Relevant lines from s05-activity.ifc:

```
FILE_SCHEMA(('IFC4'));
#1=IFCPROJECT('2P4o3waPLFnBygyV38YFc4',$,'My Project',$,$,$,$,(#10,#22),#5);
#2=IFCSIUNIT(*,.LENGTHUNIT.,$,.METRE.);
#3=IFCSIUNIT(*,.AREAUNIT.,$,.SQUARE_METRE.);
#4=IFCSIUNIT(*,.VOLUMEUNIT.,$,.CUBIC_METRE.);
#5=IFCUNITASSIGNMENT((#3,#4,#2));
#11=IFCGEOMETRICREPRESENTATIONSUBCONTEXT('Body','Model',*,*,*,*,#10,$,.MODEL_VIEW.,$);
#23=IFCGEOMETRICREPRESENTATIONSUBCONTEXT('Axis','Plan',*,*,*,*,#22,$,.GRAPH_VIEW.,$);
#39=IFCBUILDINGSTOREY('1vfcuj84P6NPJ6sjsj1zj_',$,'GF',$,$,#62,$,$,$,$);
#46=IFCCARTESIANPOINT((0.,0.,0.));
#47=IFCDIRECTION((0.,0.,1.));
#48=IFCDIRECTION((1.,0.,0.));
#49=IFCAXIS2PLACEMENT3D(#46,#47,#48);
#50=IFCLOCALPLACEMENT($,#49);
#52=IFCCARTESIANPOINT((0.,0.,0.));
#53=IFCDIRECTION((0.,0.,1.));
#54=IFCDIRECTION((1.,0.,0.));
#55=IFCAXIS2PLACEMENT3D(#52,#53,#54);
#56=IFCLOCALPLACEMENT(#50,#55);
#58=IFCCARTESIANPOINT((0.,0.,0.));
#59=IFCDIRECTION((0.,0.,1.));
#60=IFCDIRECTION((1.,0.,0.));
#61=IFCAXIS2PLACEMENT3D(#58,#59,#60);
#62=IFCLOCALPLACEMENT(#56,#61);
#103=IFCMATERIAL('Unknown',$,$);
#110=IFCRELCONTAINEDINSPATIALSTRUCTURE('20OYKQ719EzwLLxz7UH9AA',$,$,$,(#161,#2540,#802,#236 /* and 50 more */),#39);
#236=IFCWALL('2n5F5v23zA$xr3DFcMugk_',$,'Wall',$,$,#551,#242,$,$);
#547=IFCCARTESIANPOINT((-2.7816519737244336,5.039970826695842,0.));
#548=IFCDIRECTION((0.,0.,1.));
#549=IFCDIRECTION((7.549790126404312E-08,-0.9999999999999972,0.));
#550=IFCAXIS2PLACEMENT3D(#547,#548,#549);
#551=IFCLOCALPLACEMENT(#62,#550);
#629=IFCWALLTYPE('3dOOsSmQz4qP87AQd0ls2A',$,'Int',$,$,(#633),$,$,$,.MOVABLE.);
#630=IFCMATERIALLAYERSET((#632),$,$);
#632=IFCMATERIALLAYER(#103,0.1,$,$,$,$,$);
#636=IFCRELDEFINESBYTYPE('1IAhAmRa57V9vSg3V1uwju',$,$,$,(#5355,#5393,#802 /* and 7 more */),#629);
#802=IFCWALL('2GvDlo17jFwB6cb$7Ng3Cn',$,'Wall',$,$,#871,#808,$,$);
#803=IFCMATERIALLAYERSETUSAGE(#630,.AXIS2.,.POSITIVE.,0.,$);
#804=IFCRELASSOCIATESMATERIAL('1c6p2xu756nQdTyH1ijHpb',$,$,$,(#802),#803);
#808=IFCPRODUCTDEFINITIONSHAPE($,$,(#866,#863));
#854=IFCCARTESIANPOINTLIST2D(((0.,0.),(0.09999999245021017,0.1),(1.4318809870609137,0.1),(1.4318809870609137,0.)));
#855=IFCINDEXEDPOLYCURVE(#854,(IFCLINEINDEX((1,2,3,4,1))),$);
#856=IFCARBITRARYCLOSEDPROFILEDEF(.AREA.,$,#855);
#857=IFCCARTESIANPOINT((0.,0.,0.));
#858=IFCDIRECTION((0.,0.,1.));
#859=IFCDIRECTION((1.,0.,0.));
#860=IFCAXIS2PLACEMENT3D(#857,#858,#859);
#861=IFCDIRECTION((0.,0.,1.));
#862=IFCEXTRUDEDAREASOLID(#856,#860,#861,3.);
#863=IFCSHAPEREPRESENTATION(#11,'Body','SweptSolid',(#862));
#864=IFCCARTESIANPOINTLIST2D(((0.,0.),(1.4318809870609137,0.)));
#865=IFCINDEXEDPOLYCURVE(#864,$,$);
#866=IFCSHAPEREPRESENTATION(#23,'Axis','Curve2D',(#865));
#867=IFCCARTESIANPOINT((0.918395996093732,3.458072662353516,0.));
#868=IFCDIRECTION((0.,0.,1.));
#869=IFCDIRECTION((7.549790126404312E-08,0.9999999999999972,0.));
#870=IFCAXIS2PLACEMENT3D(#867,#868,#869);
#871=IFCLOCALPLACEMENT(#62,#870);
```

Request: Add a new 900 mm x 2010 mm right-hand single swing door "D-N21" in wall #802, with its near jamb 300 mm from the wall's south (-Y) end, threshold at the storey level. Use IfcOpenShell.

```python
import numpy as np
import ifcopenshell
import ifcopenshell.api.feature
import ifcopenshell.api.geometry
import ifcopenshell.api.root
import ifcopenshell.api.spatial
import ifcopenshell.geom
import ifcopenshell.util.element
import ifcopenshell.util.placement
import ifcopenshell.util.representation
import ifcopenshell.util.shape
import ifcopenshell.util.unit

model = ifcopenshell.open("s05-activity.ifc")
unit_scale = ifcopenshell.util.unit.calculate_unit_scale(model)
settings = ifcopenshell.geom.settings()


def volume(element):
    """Net volume in cubic metres, openings subtracted."""
    shape = ifcopenshell.geom.create_shape(settings, element)
    return ifcopenshell.util.shape.get_volume(shape.geometry)


wall = model.by_id(802)
storey = ifcopenshell.util.element.get_container(wall, ifc_class="IfcBuildingStorey")
context = ifcopenshell.util.representation.get_context(model, "Model", "Body", "MODEL_VIEW")
before = volume(wall)

width, height, from_end, sill = 0.9, 2.01, 0.3, 0.0  # metres

# The wall runs along its own X axis, and the end named is its -X end.
wall_shape = ifcopenshell.geom.create_shape(settings, wall)
x, y, z = ifcopenshell.util.shape.get_vertices(wall_shape.geometry).T
start = x.min() + from_end
face, thickness = float(y.min()), float(y.max() - y.min())
wall_matrix = ifcopenshell.util.placement.get_local_placement(wall.ObjectPlacement)
level = ifcopenshell.util.placement.get_local_placement(storey.ObjectPlacement)[2, 3]


def in_wall(x, y):
    """Placement at x, y metres in the wall's axes, at sill height."""
    matrix = wall_matrix.copy()
    matrix[:, 3] = wall_matrix @ np.array([x / unit_scale, y / unit_scale, 0.0, 1.0])
    matrix[2, 3] = level + sill / unit_scale
    return matrix


# Opening: a box that overshoots both wall faces by 50 mm.
opening = ifcopenshell.api.root.create_entity(model, ifc_class="IfcOpeningElement", predefined_type="OPENING")
box = ifcopenshell.api.geometry.add_wall_representation(
    model, context=context, length=width, height=height, thickness=thickness + 0.1
)
ifcopenshell.api.geometry.assign_representation(model, product=opening, representation=box)
ifcopenshell.api.geometry.edit_object_placement(model, product=opening, matrix=in_wall(start, face - 0.05), is_si=False)
ifcopenshell.api.feature.add_feature(model, feature=opening, element=wall)

door = ifcopenshell.api.root.create_entity(model, ifc_class="IfcDoor", name="D-N21", predefined_type="DOOR")
door.OverallWidth, door.OverallHeight = width / unit_scale, height / unit_scale
door.OperationType = "SINGLE_SWING_RIGHT"
body = ifcopenshell.api.geometry.add_door_representation(
    model,
    context=context,
    overall_width=door.OverallWidth,
    overall_height=door.OverallHeight,
    operation_type="SINGLE_SWING_RIGHT",
    lining_properties={"LiningDepth": thickness / unit_scale, "ThresholdDepth": thickness / unit_scale},
)
ifcopenshell.api.geometry.assign_representation(model, product=door, representation=body)
ifcopenshell.api.spatial.assign_container(model, products=[door], relating_structure=storey)
ifcopenshell.api.feature.add_filling(model, opening=opening, element=door)

# The lining spans the wall, so the door starts at the wall face.
ifcopenshell.api.geometry.edit_object_placement(model, product=door, matrix=in_wall(start, face), is_si=False)

after = volume(wall)

print(f"wall volume {before:.3f} -> {after:.3f} m3")

model.write("s05-activity_updated.ifc")
```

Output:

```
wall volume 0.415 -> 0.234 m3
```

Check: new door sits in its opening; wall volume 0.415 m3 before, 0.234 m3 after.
